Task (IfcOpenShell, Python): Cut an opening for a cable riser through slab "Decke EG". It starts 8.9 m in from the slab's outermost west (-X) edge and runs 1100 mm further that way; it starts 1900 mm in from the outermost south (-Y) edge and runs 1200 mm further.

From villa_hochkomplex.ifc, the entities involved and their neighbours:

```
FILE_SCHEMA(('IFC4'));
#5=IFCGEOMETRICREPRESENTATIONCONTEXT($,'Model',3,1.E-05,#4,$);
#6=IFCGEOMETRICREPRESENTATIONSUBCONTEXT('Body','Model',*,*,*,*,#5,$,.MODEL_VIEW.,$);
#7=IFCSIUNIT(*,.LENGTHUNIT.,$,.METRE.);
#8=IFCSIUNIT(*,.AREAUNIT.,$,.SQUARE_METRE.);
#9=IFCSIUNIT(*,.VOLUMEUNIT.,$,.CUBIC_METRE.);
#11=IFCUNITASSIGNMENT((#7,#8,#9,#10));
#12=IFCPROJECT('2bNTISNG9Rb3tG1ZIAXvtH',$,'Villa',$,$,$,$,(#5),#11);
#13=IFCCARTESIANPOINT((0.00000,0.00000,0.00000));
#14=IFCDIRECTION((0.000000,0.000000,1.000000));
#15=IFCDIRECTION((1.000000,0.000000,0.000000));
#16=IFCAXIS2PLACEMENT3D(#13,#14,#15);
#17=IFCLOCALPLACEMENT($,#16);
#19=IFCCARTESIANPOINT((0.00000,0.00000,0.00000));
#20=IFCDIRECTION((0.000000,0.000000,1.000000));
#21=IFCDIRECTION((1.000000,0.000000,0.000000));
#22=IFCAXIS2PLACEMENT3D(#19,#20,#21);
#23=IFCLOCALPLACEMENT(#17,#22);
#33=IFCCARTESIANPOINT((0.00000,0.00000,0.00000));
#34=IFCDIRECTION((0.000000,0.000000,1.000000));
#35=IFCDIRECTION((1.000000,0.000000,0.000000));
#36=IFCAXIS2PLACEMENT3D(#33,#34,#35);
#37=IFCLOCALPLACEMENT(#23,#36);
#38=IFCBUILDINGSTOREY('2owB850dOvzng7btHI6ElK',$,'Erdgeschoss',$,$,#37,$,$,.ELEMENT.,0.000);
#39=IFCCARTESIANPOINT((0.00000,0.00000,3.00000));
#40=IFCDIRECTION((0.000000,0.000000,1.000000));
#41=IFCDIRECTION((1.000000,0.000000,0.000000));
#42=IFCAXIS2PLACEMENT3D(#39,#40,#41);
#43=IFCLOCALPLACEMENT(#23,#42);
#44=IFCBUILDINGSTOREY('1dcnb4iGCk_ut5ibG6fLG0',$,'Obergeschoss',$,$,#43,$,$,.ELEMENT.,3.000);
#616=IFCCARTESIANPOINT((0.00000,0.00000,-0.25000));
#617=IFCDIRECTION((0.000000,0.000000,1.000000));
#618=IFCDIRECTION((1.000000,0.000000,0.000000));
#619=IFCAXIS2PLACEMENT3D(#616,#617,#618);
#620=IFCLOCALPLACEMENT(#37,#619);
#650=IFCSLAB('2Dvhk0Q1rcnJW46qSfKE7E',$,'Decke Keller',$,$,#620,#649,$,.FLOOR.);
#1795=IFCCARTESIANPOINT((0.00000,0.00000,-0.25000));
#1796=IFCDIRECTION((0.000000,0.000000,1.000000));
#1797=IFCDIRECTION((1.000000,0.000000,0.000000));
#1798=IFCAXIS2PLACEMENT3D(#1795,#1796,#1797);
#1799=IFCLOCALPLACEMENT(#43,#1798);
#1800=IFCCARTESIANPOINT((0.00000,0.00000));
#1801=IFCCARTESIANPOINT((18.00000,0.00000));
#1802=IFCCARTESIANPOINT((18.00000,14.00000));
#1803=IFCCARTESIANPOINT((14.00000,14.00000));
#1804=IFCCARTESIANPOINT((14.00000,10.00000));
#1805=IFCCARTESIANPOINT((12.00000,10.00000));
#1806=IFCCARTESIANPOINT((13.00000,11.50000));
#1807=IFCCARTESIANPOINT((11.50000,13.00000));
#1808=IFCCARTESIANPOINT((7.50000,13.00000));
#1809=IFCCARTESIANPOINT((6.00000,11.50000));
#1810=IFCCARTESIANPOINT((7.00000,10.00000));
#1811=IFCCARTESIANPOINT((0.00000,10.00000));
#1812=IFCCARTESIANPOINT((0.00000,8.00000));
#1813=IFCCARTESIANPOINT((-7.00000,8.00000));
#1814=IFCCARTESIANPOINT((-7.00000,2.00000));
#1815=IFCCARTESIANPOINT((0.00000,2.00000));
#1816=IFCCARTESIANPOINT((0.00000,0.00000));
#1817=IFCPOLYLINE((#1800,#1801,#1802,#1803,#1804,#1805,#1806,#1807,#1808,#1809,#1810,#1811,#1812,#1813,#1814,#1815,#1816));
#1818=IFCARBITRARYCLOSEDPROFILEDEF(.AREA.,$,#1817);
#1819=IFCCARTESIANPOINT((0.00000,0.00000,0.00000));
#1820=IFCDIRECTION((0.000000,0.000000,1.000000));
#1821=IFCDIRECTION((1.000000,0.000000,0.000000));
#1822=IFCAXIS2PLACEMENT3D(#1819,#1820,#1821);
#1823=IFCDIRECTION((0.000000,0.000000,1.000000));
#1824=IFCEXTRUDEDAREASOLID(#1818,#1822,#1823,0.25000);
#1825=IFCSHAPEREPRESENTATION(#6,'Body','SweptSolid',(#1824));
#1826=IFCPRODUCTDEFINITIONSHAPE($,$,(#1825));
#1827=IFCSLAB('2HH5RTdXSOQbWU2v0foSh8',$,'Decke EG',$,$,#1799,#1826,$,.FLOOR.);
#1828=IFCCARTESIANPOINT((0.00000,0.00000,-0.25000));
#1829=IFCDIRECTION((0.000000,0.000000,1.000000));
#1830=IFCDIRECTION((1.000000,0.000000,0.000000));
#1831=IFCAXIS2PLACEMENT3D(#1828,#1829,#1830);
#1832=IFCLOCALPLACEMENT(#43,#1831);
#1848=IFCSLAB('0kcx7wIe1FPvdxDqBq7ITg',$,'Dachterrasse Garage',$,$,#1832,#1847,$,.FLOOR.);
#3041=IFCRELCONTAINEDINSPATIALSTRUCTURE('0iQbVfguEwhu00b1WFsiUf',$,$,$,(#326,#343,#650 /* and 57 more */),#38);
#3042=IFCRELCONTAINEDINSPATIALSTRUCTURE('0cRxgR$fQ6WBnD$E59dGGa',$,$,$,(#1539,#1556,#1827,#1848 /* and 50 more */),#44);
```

```python
import numpy as np
import ifcopenshell
import ifcopenshell.api.feature
import ifcopenshell.api.geometry
import ifcopenshell.api.root
import ifcopenshell.geom
import ifcopenshell.util.placement
import ifcopenshell.util.representation
import ifcopenshell.util.shape
import ifcopenshell.util.unit

model = ifcopenshell.open("villa_hochkomplex.ifc")
unit_scale = ifcopenshell.util.unit.calculate_unit_scale(model)
settings = ifcopenshell.geom.settings()


def volume(element):
    """Net volume in cubic metres, openings subtracted."""
    shape = ifcopenshell.geom.create_shape(settings, element)
    return ifcopenshell.util.shape.get_volume(shape.geometry)


slab = model.by_guid("2HH5RTdXSOQbWU2v0foSh8")
before = volume(slab)

# Extent in the slab's own axes, in metres. The edges named are its -X and -Y sides.
slab_shape = ifcopenshell.geom.create_shape(settings, slab)
vertices = ifcopenshell.util.shape.get_vertices(slab_shape.geometry)
x_min, y_min, bottom = vertices.min(axis=0)
top = vertices[:, 2].max()

opening = ifcopenshell.api.root.create_entity(model, ifc_class="IfcOpeningElement", name="Cable riser opening", predefined_type="OPENING")
context = ifcopenshell.util.representation.get_context(model, "Model", "Body", "MODEL_VIEW")
width, depth = 1.1, 1.2
outline = [(0.0, 0.0), (width, 0.0), (width, depth), (0.0, depth), (0.0, 0.0)]
# Overshoot both faces by 50 mm so the cut is clean.
shape = ifcopenshell.api.geometry.add_slab_representation(
    model, context=context, depth=top - bottom + 0.1, polyline=outline
)
ifcopenshell.api.geometry.assign_representation(model, product=opening, representation=shape)

matrix = ifcopenshell.util.placement.get_local_placement(slab.ObjectPlacement)
matrix[:, 3] = matrix @ np.append(np.array([x_min + 8.9, y_min + 1.9, bottom - 0.05]) / unit_scale, 1.0)
ifcopenshell.api.geometry.edit_object_placement(model, product=opening, matrix=matrix, is_si=False)
ifcopenshell.api.feature.add_feature(model, feature=opening, element=slab)

after = volume(slab)

print(f"slab volume {before:.3f} -> {after:.3f} m3")

model.write("villa_hochkomplex_v2.ifc")
```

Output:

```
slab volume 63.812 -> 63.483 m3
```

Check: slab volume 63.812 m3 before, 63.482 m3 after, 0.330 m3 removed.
